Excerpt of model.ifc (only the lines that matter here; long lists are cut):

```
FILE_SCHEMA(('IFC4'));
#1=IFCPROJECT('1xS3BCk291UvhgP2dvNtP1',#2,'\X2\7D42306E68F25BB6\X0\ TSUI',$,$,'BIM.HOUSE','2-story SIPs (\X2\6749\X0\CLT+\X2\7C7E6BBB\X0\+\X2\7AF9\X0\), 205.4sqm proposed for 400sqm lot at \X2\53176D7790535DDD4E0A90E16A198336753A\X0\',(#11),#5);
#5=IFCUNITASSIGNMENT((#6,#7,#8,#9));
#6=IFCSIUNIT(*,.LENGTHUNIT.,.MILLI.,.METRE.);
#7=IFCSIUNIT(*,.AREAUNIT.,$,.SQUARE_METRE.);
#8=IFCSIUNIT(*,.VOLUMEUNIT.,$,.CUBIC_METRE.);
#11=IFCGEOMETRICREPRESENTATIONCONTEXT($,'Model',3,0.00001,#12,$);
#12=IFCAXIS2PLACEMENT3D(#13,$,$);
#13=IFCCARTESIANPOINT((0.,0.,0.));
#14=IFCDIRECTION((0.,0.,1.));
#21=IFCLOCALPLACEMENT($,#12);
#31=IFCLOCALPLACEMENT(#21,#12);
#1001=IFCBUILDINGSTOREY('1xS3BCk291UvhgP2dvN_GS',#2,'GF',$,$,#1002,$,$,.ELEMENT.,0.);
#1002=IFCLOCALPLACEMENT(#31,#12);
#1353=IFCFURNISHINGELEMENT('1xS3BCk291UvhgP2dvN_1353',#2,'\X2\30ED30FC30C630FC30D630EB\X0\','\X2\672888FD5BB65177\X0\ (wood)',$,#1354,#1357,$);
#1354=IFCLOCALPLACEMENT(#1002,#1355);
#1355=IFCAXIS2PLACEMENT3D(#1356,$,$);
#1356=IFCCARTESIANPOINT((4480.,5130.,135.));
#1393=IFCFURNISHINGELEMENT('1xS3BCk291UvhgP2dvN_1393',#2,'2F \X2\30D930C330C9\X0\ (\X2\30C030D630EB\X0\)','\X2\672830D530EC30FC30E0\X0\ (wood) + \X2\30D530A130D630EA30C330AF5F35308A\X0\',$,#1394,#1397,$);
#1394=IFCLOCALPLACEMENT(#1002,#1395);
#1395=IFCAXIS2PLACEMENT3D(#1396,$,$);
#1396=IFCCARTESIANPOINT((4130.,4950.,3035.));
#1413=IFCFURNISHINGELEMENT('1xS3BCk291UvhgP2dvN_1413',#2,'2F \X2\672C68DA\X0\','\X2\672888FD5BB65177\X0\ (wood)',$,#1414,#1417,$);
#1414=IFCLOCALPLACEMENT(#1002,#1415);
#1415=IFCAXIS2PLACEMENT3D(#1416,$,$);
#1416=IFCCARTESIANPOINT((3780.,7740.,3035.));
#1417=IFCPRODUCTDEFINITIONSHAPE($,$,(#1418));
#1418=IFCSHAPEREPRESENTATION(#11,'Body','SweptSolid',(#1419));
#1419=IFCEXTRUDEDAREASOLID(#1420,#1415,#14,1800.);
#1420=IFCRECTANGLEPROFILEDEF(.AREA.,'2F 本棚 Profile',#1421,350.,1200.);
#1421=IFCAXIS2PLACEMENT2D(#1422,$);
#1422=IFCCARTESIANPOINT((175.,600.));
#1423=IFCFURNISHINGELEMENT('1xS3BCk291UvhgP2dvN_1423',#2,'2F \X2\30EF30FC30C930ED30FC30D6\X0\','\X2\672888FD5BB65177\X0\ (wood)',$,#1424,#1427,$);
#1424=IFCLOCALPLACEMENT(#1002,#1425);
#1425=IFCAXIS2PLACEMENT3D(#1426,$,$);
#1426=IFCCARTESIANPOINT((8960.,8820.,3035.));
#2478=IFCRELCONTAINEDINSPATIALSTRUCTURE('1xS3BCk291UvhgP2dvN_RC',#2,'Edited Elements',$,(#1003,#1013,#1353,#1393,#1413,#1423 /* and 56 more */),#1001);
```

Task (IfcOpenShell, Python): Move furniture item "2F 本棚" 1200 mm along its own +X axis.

```python
import ifcopenshell
import ifcopenshell.api.geometry
import ifcopenshell.util.placement
import ifcopenshell.util.unit

model = ifcopenshell.open("model.ifc")
unit_scale = ifcopenshell.util.unit.calculate_unit_scale(model)

item = model.by_guid("1xS3BCk291UvhgP2dvN_1413")
matrix = ifcopenshell.util.placement.get_local_placement(item.ObjectPlacement)
matrix[:3, 3] += matrix[:3, 0] * 1.2 / unit_scale
ifcopenshell.api.geometry.edit_object_placement(model, product=item, matrix=matrix, is_si=False)

print(ifcopenshell.util.placement.get_local_placement(item.ObjectPlacement).round(3) + 0.0)

model.write("model_updated.ifc")
```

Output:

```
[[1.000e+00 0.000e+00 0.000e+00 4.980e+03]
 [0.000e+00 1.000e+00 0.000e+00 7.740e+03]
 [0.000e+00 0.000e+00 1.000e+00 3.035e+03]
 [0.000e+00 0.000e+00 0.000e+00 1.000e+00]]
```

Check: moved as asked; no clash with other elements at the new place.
